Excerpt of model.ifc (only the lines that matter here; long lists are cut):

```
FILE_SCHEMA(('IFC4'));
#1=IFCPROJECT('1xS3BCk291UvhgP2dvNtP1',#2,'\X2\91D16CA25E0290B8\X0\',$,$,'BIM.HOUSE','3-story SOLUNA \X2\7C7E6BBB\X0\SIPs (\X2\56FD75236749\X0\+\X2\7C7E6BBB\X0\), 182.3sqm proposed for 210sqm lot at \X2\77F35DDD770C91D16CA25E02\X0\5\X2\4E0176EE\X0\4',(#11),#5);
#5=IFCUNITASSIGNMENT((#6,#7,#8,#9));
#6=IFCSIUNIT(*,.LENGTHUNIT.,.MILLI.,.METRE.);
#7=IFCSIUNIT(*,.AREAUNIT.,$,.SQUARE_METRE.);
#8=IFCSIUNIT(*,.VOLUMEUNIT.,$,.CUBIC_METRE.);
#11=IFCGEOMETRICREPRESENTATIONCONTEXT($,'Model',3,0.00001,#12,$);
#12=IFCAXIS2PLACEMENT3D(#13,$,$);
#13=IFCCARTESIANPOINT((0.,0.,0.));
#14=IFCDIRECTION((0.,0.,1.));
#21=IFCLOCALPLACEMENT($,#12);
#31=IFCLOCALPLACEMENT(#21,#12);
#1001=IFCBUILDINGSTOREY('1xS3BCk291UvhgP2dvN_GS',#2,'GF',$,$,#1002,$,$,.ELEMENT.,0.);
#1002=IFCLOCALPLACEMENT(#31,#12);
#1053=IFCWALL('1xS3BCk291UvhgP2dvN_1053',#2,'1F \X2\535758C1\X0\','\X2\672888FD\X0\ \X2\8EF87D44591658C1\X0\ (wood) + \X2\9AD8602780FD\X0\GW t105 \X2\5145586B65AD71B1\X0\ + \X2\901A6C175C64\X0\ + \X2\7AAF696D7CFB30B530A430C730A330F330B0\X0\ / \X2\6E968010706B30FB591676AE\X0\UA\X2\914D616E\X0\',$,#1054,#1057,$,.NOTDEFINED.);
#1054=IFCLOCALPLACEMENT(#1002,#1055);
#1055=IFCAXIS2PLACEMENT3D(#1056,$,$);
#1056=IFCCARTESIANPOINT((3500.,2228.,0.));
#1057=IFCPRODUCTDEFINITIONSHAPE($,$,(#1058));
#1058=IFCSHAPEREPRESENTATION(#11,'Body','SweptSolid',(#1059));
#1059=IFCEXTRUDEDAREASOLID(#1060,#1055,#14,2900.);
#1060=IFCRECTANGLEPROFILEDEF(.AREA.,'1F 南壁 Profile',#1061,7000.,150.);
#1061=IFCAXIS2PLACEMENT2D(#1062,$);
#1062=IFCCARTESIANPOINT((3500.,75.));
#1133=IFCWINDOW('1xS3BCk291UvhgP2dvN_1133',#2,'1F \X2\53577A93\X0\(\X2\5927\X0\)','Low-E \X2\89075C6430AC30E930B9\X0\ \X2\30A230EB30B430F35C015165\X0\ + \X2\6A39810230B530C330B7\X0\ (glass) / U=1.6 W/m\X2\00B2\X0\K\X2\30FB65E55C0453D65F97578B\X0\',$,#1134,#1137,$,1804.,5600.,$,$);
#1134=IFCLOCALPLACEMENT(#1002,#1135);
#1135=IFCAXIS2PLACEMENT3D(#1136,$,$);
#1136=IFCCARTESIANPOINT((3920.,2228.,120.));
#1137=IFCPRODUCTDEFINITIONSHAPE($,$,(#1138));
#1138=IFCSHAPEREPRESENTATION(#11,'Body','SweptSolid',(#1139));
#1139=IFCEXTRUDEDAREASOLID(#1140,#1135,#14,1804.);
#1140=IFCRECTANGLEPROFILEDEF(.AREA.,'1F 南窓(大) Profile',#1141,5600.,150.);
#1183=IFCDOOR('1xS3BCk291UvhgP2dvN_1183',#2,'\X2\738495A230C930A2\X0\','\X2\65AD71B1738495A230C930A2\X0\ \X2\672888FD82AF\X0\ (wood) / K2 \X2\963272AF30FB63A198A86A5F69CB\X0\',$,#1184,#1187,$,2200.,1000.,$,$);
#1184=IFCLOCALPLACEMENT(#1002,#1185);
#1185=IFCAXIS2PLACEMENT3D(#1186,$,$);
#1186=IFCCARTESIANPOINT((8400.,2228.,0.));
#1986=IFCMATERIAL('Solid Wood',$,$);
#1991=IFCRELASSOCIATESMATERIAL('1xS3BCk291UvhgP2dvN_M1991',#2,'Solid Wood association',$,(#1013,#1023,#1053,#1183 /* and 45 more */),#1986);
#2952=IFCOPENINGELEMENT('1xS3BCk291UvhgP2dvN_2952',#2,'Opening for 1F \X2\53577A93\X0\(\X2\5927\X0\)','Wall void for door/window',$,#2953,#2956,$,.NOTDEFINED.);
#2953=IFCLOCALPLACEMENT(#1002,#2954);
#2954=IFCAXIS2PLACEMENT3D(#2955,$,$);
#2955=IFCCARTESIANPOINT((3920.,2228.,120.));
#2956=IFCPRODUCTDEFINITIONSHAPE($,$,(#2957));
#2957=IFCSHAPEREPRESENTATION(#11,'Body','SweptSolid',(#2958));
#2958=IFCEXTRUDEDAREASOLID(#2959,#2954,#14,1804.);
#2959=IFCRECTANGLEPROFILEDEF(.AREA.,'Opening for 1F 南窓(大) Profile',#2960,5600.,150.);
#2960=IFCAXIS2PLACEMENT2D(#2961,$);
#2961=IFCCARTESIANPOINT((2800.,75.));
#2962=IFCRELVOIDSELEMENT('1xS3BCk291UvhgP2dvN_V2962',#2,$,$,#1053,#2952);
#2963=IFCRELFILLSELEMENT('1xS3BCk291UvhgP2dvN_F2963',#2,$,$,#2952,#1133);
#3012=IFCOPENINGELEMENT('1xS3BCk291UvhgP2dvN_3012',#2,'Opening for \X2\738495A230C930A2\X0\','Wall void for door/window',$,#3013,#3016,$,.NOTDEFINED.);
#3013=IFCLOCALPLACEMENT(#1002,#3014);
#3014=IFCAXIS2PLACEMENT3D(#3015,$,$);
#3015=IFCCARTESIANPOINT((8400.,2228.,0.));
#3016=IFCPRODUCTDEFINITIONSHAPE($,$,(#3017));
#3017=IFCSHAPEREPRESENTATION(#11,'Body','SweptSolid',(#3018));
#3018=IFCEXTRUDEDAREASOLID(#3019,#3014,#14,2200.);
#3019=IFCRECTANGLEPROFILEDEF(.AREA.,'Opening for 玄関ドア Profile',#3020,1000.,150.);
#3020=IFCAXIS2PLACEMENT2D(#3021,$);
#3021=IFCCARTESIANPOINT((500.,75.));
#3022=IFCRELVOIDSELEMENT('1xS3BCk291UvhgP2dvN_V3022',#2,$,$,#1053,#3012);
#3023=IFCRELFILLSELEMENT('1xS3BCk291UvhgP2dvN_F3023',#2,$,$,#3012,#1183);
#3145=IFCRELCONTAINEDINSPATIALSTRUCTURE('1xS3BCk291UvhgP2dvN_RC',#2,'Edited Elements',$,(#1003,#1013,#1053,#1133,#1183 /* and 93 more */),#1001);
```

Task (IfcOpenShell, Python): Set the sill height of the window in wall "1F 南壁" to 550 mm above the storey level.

```python
import numpy as np
import ifcopenshell
import ifcopenshell.api.geometry
import ifcopenshell.geom
import ifcopenshell.util.element
import ifcopenshell.util.placement
import ifcopenshell.util.shape
import ifcopenshell.util.unit

model = ifcopenshell.open("model.ifc")
unit_scale = ifcopenshell.util.unit.calculate_unit_scale(model)

window = model.by_guid("1xS3BCk291UvhgP2dvN_1133")
opening = window.FillsVoids[0].RelatingOpeningElement
storey = ifcopenshell.util.element.get_container(window, ifc_class="IfcBuildingStorey")
level = ifcopenshell.util.placement.get_local_placement(storey.ObjectPlacement)[2, 3]

# The opening's origin need not be at the sill, so measure its lowest point.
shape = ifcopenshell.geom.create_shape(ifcopenshell.geom.settings(), opening)
bottom = ifcopenshell.util.shape.get_shape_bottom_elevation(shape, shape.geometry) / unit_scale
dz = level + 550.0 - bottom

shift = np.array([0.0, 0.0, dz])
# The window is not placed relative to its opening, so move both.
for product in (opening, window):
    matrix = ifcopenshell.util.placement.get_local_placement(product.ObjectPlacement)
    matrix[:3, 3] += shift
    ifcopenshell.api.geometry.edit_object_placement(model, product=product, matrix=matrix, is_si=False)

print(f"moved by {dz * unit_scale:+.3f} m")

model.write("model_v2.ifc")
```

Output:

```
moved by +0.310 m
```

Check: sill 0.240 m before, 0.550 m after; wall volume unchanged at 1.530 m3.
